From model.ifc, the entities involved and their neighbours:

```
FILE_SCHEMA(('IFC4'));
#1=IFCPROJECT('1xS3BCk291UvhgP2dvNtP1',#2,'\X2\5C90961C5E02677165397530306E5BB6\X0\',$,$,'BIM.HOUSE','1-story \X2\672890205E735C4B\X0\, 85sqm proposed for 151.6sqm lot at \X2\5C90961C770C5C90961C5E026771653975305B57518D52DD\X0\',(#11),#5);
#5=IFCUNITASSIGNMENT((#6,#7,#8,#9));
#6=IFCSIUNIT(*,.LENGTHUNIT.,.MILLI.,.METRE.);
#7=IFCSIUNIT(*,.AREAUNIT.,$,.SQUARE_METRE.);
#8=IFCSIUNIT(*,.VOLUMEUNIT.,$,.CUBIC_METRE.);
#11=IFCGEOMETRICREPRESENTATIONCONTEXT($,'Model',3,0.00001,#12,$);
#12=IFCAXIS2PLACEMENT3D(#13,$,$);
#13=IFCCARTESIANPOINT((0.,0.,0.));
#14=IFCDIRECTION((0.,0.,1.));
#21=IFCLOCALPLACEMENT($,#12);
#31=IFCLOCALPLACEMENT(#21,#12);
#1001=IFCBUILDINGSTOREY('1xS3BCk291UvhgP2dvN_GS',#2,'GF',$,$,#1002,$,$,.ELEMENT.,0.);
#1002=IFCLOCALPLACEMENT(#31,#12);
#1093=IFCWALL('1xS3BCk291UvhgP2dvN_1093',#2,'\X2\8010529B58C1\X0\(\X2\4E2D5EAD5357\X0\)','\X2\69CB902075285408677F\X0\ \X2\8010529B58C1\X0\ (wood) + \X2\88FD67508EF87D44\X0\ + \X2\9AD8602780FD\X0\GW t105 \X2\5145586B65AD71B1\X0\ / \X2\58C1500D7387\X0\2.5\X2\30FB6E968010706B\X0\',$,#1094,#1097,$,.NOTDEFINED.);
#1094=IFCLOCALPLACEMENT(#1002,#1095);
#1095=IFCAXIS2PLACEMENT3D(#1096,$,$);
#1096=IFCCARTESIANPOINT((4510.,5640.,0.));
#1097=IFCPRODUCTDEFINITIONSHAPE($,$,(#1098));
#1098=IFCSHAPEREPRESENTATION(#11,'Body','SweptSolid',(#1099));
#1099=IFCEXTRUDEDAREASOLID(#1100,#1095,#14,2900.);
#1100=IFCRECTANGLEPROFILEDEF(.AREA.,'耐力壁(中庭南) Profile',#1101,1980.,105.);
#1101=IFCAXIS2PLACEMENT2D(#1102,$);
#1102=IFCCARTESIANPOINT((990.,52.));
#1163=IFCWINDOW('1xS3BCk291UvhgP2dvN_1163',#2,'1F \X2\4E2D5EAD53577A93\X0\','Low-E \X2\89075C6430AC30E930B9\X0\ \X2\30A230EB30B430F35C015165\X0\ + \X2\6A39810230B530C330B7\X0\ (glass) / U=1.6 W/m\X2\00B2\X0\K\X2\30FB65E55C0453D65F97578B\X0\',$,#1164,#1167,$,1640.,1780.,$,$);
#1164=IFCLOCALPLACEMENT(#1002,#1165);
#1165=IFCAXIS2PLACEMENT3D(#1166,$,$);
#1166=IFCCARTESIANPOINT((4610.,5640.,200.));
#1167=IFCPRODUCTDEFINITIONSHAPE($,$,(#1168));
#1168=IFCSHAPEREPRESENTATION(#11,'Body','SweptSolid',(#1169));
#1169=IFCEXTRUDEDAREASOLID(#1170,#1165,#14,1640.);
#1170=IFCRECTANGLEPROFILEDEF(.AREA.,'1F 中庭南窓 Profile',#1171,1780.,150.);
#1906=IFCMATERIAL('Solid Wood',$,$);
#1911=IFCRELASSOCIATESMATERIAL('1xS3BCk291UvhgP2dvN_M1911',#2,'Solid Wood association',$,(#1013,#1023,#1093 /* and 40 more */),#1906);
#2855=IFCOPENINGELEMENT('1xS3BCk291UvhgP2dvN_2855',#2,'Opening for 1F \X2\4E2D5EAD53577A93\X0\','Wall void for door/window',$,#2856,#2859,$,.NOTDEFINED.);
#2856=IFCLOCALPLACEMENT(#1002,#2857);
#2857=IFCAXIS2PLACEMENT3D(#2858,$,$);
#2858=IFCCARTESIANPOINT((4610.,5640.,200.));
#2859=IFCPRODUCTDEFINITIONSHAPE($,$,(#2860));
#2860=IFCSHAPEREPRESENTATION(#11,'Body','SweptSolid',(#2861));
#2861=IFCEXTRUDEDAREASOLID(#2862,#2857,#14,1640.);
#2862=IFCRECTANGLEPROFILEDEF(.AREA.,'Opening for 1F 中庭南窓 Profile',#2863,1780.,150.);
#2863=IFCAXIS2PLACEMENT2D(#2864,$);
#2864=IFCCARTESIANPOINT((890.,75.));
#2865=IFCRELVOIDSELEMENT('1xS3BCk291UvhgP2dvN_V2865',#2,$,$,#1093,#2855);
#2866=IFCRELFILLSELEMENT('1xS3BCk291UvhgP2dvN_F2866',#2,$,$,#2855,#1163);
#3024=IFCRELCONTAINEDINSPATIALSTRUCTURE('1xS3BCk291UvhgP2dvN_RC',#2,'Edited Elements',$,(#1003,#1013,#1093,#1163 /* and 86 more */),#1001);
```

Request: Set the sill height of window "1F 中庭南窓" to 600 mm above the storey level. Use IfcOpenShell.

```python
import numpy as np
import ifcopenshell
import ifcopenshell.api.geometry
import ifcopenshell.geom
import ifcopenshell.util.element
import ifcopenshell.util.placement
import ifcopenshell.util.shape
import ifcopenshell.util.unit

model = ifcopenshell.open("model.ifc")
unit_scale = ifcopenshell.util.unit.calculate_unit_scale(model)

window = model.by_guid("1xS3BCk291UvhgP2dvN_1163")
opening = window.FillsVoids[0].RelatingOpeningElement
storey = ifcopenshell.util.element.get_container(window, ifc_class="IfcBuildingStorey")
level = ifcopenshell.util.placement.get_local_placement(storey.ObjectPlacement)[2, 3]

# The opening's origin need not be at the sill, so measure its lowest point.
shape = ifcopenshell.geom.create_shape(ifcopenshell.geom.settings(), opening)
bottom = ifcopenshell.util.shape.get_shape_bottom_elevation(shape, shape.geometry) / unit_scale
dz = level + 0.6 / unit_scale - bottom

shift = np.array([0.0, 0.0, dz])
# The window is not placed relative to its opening, so move both.
for product in (opening, window):
    matrix = ifcopenshell.util.placement.get_local_placement(product.ObjectPlacement)
    matrix[:3, 3] += shift
    ifcopenshell.api.geometry.edit_object_placement(model, product=product, matrix=matrix, is_si=False)

print(f"moved by {dz * unit_scale:+.3f} m")

model.write("model_rev.ifc")
```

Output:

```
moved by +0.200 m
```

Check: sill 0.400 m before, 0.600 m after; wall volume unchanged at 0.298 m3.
